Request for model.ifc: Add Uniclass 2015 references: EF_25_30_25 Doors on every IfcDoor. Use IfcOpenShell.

First a look at what the model holds.

```python
import ifcopenshell

model = ifcopenshell.open("model.ifc")
print(model.schema)
print("classifications:", [c.Name for c in model.by_type("IfcClassification")])
for ifc_class in ("IfcDoor", "IfcRoof", "IfcStair", "IfcWall", "IfcWindow"):
    print(ifc_class, len(model.by_type(ifc_class)))
```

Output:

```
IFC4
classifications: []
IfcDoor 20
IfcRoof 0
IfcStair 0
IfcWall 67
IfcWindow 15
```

```python
import ifcopenshell
import ifcopenshell.api.classification

model = ifcopenshell.open("model.ifc")

system = ifcopenshell.api.classification.add_classification(model, classification="Uniclass 2015")

codes = {
    "IfcDoor": ("EF_25_30_25", "Doors"),
}
for ifc_class, (code, name) in codes.items():
    products = model.by_type(ifc_class)
    ifcopenshell.api.classification.add_reference(
        model, products=products, classification=system, identification=code, name=name
    )
    print(code, len(products))

model.write("model_v2.ifc")
```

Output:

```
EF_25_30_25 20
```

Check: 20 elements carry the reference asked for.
